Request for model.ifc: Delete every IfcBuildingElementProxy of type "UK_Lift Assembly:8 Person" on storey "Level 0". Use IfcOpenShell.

First a look at what the model holds.

```python
import ifcopenshell
import ifcopenshell.util.element

model = ifcopenshell.open("model.ifc")
print(model.schema)
storey = next(s for s in model.by_type("IfcBuildingStorey") if s.Name == "Level 0")
proxies = [e for e in ifcopenshell.util.element.get_decomposition(storey) if e.is_a("IfcBuildingElementProxy")]
seen = {}
for e in proxies:
    element_type = ifcopenshell.util.element.get_type(e)
    name = element_type.Name if element_type not in (None, e) else None
    seen[name] = seen.get(name, 0) + 1
for name, count in sorted(seen.items(), key=str):
    print(count, "x", name)
```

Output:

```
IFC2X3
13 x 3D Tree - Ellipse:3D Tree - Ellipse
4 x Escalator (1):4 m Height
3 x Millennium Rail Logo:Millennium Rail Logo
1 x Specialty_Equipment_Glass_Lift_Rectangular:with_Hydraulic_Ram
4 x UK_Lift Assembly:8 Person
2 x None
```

```python
import ifcopenshell
import ifcopenshell.api.root
import ifcopenshell.util.element

model = ifcopenshell.open("model.ifc")

storey = next(s for s in model.by_type("IfcBuildingStorey") if s.Name == "Level 0")
proxies = [e for e in ifcopenshell.util.element.get_decomposition(storey) if e.is_a("IfcBuildingElementProxy")]
targets = [e for e in proxies if (t := ifcopenshell.util.element.get_type(e)) not in (None, e) and t.Name == "UK_Lift Assembly:8 Person"]

for e in targets:
    ifcopenshell.api.root.remove_product(model, product=e)
print(len(targets), "removed")

model.write("model_updated.ifc")
```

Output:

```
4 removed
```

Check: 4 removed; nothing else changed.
